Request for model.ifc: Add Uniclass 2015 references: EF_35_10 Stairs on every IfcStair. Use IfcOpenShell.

First a look at what the model holds.

```python
import ifcopenshell

model = ifcopenshell.open("model.ifc")
print(model.schema)
print("classifications:", [c.Name for c in model.by_type("IfcClassification")])
for ifc_class in ("IfcDoor", "IfcRoof", "IfcStair", "IfcWall", "IfcWindow"):
    print(ifc_class, len(model.by_type(ifc_class)))
```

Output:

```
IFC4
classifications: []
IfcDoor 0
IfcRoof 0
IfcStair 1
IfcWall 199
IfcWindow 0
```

```python
import ifcopenshell
import ifcopenshell.api.classification

model = ifcopenshell.open("model.ifc")

system = ifcopenshell.api.classification.add_classification(model, classification="Uniclass 2015")

codes = {
    "IfcStair": ("EF_35_10", "Stairs"),
}
for ifc_class, (code, name) in codes.items():
    products = model.by_type(ifc_class)
    ifcopenshell.api.classification.add_reference(
        model, products=products, classification=system, identification=code, name=name
    )
    print(code, len(products))

model.write("model_updated.ifc")
```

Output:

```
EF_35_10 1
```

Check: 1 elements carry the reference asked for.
